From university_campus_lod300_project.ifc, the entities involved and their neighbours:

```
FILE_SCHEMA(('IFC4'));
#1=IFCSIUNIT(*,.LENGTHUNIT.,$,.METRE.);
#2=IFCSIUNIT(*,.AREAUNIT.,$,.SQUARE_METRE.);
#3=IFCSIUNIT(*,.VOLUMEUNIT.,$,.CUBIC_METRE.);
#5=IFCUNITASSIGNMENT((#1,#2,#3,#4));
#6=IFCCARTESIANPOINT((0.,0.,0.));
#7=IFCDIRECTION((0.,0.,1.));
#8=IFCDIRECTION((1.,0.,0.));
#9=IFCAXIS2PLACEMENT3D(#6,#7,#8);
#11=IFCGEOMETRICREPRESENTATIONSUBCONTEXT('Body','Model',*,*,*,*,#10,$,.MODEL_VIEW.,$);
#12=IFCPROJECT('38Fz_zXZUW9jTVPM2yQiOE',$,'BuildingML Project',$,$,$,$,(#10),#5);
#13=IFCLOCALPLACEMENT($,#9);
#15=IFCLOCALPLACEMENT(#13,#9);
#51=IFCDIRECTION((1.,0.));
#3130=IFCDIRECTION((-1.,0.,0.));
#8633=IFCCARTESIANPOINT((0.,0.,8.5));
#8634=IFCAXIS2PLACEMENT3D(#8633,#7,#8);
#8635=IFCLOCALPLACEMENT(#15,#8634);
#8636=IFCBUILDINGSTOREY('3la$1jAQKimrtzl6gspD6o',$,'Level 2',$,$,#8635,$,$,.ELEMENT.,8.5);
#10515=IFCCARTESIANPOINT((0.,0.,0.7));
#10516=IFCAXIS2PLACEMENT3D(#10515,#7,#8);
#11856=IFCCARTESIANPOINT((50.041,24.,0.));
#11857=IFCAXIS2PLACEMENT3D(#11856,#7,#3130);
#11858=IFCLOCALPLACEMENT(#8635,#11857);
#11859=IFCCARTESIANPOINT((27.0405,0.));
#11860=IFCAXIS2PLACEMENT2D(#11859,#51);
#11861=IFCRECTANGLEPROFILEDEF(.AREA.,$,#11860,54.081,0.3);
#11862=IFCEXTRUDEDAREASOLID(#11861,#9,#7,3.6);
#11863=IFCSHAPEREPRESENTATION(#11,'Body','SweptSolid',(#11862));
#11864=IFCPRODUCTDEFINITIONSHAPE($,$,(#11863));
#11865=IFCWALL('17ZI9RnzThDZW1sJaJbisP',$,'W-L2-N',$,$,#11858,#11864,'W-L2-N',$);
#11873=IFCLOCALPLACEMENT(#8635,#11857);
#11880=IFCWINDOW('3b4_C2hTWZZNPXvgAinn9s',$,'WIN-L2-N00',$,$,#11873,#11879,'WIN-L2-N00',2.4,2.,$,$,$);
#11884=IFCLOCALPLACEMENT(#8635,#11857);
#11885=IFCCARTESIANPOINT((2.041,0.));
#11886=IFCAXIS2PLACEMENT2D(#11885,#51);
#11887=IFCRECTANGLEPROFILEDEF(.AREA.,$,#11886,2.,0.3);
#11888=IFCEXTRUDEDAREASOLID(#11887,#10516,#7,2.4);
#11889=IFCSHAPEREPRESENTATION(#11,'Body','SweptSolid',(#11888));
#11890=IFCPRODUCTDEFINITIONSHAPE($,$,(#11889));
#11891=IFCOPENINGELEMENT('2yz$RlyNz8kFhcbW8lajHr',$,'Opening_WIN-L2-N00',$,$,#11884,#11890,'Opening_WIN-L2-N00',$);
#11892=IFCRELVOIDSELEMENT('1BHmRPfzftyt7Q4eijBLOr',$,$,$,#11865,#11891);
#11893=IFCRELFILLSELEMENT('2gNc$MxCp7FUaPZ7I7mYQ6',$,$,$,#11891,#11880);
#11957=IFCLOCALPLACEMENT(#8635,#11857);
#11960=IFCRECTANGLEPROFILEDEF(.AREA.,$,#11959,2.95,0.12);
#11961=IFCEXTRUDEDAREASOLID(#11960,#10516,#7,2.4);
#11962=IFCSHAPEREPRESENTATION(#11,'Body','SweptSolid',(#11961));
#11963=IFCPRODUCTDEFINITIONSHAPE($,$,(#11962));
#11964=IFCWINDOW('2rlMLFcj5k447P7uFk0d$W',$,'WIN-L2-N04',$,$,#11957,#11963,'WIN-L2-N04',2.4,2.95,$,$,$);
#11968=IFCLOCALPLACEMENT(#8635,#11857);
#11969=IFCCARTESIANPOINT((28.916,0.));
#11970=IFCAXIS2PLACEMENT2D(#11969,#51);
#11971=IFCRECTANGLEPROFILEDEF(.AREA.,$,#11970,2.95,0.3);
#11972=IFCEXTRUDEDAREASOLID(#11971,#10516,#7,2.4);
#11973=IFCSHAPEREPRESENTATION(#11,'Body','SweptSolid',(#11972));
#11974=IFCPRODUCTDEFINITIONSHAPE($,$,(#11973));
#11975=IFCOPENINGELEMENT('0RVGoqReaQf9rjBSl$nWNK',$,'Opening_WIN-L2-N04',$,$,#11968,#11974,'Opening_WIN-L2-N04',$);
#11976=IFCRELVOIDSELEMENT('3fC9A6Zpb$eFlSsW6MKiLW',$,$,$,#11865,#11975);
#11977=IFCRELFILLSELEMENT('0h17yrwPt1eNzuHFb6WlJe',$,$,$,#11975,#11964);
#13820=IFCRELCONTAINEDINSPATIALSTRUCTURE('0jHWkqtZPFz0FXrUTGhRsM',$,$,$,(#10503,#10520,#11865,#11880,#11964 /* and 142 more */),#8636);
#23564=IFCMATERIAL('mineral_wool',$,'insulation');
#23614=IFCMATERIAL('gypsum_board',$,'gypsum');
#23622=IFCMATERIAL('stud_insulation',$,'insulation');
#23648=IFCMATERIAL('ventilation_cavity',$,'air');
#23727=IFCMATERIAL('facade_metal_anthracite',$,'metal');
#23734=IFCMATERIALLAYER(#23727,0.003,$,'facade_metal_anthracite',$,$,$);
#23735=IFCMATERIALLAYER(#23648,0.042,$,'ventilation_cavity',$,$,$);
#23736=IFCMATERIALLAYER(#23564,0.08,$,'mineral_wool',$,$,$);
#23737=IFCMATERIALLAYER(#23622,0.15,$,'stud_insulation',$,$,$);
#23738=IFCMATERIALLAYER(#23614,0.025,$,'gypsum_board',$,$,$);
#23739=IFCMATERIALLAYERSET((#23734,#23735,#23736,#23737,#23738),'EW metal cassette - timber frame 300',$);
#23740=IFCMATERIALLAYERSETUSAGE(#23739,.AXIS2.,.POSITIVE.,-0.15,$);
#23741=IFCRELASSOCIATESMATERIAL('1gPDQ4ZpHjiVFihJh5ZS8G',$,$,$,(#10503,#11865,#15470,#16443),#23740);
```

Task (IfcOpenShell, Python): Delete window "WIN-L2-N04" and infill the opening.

```python
import ifcopenshell
import ifcopenshell.api.feature
import ifcopenshell.api.root
import ifcopenshell.geom
import ifcopenshell.util.shape

model = ifcopenshell.open("university_campus_lod300_project.ifc")
settings = ifcopenshell.geom.settings()


def volume(element):
    """Net volume in cubic metres, openings subtracted."""
    shape = ifcopenshell.geom.create_shape(settings, element)
    return ifcopenshell.util.shape.get_volume(shape.geometry)


window = model.by_guid("2rlMLFcj5k447P7uFk0d$W")
opening = window.FillsVoids[0].RelatingOpeningElement
wall = opening.VoidsElements[0].RelatingBuildingElement
before = volume(wall)

ifcopenshell.api.root.remove_product(model, product=window)
ifcopenshell.api.feature.remove_feature(model, feature=opening)

after = volume(wall)

print(f"wall volume {before:.3f} -> {after:.3f} m3")

model.write("university_campus_lod300_project-out.ifc")
```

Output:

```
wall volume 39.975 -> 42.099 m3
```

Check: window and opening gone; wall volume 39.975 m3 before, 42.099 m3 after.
